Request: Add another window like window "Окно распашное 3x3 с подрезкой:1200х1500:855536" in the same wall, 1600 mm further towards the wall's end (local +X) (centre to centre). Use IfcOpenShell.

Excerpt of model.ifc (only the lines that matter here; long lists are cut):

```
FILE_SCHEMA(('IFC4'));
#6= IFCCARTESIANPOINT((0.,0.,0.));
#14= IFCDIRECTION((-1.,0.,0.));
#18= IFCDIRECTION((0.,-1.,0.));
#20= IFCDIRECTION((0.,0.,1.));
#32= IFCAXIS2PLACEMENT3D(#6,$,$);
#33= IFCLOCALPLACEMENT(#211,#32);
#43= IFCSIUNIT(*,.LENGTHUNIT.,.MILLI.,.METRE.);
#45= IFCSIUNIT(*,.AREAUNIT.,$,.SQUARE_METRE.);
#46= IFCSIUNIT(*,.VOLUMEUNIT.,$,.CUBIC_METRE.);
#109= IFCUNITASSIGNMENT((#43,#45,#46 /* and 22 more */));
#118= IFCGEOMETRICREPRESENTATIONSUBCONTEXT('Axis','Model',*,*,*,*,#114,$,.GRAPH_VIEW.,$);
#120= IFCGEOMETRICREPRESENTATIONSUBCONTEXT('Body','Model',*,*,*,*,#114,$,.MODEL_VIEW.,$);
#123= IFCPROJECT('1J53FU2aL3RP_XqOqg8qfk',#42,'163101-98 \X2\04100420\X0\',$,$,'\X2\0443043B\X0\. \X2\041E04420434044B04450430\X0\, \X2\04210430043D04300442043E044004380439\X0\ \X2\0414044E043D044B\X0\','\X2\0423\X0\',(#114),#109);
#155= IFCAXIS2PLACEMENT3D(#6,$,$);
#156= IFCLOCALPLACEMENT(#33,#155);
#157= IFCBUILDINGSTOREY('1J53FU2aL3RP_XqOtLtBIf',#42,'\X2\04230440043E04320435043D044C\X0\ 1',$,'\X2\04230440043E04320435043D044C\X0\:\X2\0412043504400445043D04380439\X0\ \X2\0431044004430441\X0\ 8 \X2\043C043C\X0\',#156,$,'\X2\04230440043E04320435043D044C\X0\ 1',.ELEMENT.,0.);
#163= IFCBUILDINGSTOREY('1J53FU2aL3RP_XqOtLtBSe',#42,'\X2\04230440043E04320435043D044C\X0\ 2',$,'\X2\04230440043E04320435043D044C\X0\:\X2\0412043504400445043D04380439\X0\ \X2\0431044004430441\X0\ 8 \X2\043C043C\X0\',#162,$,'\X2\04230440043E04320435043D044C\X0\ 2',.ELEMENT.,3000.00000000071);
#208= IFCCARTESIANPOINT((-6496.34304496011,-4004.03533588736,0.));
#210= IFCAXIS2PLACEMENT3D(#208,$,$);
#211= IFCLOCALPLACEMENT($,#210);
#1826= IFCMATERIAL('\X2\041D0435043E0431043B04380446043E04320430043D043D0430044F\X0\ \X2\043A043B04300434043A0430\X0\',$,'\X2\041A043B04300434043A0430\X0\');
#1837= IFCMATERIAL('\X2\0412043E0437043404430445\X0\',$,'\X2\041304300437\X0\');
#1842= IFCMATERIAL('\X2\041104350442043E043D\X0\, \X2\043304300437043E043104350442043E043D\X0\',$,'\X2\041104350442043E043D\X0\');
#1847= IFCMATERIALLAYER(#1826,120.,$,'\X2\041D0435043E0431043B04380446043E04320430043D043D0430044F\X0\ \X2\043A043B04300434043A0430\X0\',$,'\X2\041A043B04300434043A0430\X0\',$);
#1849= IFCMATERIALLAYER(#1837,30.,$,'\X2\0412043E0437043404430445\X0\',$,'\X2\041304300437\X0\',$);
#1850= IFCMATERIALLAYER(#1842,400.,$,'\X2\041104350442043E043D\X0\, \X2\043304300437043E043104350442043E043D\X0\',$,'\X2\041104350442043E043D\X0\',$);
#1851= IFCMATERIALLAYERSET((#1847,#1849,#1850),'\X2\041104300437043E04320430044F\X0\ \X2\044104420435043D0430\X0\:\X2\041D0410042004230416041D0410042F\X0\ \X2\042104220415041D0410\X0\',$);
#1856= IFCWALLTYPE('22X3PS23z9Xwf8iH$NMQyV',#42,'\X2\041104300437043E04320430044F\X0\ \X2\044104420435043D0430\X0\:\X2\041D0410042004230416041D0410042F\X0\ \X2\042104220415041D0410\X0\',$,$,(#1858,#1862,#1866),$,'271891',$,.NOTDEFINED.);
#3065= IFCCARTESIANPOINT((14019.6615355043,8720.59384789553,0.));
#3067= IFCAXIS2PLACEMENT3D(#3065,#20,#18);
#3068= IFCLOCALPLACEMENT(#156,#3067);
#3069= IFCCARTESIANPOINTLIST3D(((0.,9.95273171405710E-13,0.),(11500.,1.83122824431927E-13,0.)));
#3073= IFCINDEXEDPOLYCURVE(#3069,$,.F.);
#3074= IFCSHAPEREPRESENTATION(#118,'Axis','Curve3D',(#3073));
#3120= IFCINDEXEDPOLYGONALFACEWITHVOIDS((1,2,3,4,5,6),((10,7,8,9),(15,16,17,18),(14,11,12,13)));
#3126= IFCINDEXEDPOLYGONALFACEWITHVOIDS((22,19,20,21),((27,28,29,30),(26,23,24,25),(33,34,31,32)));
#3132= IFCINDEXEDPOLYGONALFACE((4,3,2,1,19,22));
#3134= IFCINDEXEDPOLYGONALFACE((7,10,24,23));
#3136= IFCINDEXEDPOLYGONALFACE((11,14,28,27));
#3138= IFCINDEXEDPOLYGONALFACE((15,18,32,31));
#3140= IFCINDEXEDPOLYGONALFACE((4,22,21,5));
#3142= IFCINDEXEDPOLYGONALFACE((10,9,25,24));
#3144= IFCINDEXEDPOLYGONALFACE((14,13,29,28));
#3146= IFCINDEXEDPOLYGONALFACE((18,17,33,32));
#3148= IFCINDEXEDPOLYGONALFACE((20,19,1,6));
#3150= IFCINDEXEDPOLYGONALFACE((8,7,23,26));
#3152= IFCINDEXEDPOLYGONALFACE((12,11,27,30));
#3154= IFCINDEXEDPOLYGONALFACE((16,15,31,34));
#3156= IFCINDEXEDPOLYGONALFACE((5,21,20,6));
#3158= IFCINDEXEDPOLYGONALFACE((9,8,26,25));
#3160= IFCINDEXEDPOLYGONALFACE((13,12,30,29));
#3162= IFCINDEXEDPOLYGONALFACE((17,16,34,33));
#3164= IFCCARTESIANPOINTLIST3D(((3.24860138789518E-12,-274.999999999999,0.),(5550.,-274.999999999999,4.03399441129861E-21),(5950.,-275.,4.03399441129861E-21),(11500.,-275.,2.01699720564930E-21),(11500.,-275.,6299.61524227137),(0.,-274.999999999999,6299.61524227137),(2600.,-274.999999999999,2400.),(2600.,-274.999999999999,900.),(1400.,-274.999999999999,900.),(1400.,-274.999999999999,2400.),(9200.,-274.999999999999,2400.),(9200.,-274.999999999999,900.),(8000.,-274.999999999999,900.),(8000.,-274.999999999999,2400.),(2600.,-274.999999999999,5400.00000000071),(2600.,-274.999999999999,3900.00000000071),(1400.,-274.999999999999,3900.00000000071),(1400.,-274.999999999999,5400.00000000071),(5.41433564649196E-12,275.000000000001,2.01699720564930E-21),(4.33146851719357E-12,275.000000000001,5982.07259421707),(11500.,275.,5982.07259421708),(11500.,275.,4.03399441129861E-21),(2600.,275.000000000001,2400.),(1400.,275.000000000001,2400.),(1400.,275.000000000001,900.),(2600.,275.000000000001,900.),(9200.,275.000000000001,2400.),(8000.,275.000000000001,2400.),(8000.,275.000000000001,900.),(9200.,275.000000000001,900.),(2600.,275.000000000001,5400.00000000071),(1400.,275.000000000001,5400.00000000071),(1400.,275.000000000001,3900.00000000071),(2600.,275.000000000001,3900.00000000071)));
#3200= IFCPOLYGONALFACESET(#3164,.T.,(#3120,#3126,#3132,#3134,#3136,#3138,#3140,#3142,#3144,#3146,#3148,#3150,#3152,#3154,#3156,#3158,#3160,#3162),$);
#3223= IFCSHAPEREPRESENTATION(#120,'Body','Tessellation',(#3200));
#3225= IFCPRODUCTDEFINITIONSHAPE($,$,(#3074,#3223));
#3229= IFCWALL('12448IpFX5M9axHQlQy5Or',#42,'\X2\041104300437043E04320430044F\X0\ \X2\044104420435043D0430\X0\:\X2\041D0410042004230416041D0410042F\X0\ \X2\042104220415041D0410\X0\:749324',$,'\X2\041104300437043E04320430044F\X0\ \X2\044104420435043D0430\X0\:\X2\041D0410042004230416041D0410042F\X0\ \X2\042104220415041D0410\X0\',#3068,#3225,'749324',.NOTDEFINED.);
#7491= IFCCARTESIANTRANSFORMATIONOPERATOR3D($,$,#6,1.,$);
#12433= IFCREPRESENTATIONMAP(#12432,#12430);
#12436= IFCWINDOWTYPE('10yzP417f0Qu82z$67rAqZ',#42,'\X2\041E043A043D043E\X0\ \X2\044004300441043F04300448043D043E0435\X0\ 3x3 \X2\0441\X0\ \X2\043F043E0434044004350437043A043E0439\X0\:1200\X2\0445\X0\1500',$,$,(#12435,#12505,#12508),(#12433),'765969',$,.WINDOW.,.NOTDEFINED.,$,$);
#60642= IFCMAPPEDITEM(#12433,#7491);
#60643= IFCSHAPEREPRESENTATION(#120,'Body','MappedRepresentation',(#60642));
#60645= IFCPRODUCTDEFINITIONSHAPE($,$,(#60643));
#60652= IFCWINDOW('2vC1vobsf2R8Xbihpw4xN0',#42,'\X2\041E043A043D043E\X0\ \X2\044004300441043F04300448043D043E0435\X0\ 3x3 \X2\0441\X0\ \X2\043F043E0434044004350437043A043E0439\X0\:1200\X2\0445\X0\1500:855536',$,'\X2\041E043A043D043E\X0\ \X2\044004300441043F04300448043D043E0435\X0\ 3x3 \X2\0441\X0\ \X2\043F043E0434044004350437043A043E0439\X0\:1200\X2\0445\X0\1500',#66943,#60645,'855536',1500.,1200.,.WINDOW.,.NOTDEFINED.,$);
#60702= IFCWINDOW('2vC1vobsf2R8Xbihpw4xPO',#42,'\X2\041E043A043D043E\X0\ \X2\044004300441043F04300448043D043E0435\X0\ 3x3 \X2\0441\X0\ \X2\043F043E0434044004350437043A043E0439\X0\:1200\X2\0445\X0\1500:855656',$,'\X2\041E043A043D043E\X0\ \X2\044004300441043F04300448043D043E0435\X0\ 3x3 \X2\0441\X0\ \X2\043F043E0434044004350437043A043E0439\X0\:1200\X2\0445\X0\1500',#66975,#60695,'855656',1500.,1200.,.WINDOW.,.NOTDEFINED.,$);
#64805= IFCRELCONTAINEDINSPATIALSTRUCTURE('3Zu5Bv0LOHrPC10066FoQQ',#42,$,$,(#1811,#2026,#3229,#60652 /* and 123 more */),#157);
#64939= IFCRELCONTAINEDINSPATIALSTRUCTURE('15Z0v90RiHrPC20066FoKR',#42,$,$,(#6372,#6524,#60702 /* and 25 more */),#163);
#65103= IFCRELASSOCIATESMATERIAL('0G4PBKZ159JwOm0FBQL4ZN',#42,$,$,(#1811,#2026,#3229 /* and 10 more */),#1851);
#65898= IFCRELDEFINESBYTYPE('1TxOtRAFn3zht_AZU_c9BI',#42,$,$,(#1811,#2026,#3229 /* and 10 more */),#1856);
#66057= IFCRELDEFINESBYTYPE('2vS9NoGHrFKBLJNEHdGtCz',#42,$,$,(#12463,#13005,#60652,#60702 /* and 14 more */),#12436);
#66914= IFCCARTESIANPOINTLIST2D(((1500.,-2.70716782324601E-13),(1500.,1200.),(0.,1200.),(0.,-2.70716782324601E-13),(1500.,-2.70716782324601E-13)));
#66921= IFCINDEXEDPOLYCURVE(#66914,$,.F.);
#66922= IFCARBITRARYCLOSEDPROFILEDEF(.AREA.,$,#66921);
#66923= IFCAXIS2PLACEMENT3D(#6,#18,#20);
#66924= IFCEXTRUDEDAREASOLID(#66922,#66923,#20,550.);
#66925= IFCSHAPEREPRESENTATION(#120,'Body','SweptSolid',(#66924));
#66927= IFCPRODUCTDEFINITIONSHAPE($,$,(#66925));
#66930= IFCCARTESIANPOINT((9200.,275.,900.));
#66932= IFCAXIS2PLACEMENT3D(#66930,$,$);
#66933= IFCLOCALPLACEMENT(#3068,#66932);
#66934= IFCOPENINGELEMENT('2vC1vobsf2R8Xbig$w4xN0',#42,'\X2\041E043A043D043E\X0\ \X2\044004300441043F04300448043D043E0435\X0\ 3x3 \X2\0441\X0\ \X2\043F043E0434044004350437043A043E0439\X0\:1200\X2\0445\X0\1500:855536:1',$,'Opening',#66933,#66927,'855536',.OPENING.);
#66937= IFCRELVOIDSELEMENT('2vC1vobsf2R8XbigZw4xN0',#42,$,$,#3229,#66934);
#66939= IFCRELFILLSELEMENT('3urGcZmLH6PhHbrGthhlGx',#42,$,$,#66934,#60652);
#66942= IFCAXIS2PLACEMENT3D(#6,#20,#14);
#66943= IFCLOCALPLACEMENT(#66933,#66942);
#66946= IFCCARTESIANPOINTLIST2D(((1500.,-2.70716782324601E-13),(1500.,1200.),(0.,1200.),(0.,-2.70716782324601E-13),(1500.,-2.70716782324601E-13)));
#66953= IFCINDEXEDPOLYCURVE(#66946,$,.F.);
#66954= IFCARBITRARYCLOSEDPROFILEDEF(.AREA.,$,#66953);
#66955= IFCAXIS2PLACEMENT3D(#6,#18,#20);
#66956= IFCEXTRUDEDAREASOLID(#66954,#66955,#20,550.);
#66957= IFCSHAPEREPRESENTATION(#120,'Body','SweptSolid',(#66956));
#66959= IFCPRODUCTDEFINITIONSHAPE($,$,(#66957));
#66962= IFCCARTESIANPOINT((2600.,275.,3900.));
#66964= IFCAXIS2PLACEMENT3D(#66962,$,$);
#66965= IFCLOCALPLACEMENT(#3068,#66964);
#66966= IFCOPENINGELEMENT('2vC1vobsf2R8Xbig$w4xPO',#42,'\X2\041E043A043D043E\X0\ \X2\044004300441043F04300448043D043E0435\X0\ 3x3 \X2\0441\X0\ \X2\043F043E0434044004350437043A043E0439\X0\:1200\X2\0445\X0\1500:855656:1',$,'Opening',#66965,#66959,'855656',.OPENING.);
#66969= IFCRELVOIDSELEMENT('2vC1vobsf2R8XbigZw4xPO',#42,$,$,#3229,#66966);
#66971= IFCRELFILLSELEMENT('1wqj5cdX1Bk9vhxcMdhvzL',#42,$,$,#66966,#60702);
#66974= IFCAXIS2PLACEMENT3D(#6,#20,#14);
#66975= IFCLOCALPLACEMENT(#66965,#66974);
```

```python
import ifcopenshell
import ifcopenshell.api.feature
import ifcopenshell.api.geometry
import ifcopenshell.api.root
import ifcopenshell.geom
import ifcopenshell.util.element
import ifcopenshell.util.placement
import ifcopenshell.util.shape
import ifcopenshell.util.unit

model = ifcopenshell.open("model.ifc")
unit_scale = ifcopenshell.util.unit.calculate_unit_scale(model)
settings = ifcopenshell.geom.settings()


def volume(element):
    """Net volume in cubic metres, openings subtracted."""
    shape = ifcopenshell.geom.create_shape(settings, element)
    return ifcopenshell.util.shape.get_volume(shape.geometry)


def reuse_history(source, copy):
    """copy_class also copies each property set's owner history, people and application; keep the originals."""
    for rel in copy.IsDefinedBy:
        if rel.is_a("IfcRelDefinesByProperties") and (history := rel.RelatingPropertyDefinition.OwnerHistory):
            rel.RelatingPropertyDefinition.OwnerHistory = source.OwnerHistory
            ifcopenshell.util.element.remove_deep2(model, history)


window = model.by_guid("2vC1vobsf2R8Xbihpw4xN0")
opening = window.FillsVoids[0].RelatingOpeningElement
wall = opening.VoidsElements[0].RelatingBuildingElement
before = volume(wall)
shift = ifcopenshell.util.placement.get_local_placement(wall.ObjectPlacement)[:3, 0] * 1.6 / unit_scale

# copy_class copies the void relationship, type, container and properties, but no geometry.
new_opening = ifcopenshell.api.root.copy_class(model, product=opening)
new_opening.Representation = ifcopenshell.util.element.copy_deep(
    model, opening.Representation, exclude=["IfcGeometricRepresentationContext", "IfcRepresentationMap"]
)
new_opening.Name = "Окно распашное 3x3 с подрезкой:1200х1500"
new_opening.Tag = None
new_window = ifcopenshell.api.root.copy_class(model, product=window)
new_window.Representation = ifcopenshell.util.element.copy_deep(
    model, window.Representation, exclude=["IfcGeometricRepresentationContext", "IfcRepresentationMap"]
)
new_window.Name = "Окно распашное 3x3 с подрезкой:1200х1500"
new_window.Tag = None
reuse_history(window, new_window)
ifcopenshell.api.feature.add_filling(model, opening=new_opening, element=new_window)

for old, new in ((opening, new_opening), (window, new_window)):
    matrix = ifcopenshell.util.placement.get_local_placement(old.ObjectPlacement)
    matrix[:3, 3] += shift
    ifcopenshell.api.geometry.edit_object_placement(model, product=new, matrix=matrix, is_si=False)

after = volume(wall)

print(f"wall volume {before:.3f} -> {after:.3f} m3")

model.write("model_rev.ifc")
```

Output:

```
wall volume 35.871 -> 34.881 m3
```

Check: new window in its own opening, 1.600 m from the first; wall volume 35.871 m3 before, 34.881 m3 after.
